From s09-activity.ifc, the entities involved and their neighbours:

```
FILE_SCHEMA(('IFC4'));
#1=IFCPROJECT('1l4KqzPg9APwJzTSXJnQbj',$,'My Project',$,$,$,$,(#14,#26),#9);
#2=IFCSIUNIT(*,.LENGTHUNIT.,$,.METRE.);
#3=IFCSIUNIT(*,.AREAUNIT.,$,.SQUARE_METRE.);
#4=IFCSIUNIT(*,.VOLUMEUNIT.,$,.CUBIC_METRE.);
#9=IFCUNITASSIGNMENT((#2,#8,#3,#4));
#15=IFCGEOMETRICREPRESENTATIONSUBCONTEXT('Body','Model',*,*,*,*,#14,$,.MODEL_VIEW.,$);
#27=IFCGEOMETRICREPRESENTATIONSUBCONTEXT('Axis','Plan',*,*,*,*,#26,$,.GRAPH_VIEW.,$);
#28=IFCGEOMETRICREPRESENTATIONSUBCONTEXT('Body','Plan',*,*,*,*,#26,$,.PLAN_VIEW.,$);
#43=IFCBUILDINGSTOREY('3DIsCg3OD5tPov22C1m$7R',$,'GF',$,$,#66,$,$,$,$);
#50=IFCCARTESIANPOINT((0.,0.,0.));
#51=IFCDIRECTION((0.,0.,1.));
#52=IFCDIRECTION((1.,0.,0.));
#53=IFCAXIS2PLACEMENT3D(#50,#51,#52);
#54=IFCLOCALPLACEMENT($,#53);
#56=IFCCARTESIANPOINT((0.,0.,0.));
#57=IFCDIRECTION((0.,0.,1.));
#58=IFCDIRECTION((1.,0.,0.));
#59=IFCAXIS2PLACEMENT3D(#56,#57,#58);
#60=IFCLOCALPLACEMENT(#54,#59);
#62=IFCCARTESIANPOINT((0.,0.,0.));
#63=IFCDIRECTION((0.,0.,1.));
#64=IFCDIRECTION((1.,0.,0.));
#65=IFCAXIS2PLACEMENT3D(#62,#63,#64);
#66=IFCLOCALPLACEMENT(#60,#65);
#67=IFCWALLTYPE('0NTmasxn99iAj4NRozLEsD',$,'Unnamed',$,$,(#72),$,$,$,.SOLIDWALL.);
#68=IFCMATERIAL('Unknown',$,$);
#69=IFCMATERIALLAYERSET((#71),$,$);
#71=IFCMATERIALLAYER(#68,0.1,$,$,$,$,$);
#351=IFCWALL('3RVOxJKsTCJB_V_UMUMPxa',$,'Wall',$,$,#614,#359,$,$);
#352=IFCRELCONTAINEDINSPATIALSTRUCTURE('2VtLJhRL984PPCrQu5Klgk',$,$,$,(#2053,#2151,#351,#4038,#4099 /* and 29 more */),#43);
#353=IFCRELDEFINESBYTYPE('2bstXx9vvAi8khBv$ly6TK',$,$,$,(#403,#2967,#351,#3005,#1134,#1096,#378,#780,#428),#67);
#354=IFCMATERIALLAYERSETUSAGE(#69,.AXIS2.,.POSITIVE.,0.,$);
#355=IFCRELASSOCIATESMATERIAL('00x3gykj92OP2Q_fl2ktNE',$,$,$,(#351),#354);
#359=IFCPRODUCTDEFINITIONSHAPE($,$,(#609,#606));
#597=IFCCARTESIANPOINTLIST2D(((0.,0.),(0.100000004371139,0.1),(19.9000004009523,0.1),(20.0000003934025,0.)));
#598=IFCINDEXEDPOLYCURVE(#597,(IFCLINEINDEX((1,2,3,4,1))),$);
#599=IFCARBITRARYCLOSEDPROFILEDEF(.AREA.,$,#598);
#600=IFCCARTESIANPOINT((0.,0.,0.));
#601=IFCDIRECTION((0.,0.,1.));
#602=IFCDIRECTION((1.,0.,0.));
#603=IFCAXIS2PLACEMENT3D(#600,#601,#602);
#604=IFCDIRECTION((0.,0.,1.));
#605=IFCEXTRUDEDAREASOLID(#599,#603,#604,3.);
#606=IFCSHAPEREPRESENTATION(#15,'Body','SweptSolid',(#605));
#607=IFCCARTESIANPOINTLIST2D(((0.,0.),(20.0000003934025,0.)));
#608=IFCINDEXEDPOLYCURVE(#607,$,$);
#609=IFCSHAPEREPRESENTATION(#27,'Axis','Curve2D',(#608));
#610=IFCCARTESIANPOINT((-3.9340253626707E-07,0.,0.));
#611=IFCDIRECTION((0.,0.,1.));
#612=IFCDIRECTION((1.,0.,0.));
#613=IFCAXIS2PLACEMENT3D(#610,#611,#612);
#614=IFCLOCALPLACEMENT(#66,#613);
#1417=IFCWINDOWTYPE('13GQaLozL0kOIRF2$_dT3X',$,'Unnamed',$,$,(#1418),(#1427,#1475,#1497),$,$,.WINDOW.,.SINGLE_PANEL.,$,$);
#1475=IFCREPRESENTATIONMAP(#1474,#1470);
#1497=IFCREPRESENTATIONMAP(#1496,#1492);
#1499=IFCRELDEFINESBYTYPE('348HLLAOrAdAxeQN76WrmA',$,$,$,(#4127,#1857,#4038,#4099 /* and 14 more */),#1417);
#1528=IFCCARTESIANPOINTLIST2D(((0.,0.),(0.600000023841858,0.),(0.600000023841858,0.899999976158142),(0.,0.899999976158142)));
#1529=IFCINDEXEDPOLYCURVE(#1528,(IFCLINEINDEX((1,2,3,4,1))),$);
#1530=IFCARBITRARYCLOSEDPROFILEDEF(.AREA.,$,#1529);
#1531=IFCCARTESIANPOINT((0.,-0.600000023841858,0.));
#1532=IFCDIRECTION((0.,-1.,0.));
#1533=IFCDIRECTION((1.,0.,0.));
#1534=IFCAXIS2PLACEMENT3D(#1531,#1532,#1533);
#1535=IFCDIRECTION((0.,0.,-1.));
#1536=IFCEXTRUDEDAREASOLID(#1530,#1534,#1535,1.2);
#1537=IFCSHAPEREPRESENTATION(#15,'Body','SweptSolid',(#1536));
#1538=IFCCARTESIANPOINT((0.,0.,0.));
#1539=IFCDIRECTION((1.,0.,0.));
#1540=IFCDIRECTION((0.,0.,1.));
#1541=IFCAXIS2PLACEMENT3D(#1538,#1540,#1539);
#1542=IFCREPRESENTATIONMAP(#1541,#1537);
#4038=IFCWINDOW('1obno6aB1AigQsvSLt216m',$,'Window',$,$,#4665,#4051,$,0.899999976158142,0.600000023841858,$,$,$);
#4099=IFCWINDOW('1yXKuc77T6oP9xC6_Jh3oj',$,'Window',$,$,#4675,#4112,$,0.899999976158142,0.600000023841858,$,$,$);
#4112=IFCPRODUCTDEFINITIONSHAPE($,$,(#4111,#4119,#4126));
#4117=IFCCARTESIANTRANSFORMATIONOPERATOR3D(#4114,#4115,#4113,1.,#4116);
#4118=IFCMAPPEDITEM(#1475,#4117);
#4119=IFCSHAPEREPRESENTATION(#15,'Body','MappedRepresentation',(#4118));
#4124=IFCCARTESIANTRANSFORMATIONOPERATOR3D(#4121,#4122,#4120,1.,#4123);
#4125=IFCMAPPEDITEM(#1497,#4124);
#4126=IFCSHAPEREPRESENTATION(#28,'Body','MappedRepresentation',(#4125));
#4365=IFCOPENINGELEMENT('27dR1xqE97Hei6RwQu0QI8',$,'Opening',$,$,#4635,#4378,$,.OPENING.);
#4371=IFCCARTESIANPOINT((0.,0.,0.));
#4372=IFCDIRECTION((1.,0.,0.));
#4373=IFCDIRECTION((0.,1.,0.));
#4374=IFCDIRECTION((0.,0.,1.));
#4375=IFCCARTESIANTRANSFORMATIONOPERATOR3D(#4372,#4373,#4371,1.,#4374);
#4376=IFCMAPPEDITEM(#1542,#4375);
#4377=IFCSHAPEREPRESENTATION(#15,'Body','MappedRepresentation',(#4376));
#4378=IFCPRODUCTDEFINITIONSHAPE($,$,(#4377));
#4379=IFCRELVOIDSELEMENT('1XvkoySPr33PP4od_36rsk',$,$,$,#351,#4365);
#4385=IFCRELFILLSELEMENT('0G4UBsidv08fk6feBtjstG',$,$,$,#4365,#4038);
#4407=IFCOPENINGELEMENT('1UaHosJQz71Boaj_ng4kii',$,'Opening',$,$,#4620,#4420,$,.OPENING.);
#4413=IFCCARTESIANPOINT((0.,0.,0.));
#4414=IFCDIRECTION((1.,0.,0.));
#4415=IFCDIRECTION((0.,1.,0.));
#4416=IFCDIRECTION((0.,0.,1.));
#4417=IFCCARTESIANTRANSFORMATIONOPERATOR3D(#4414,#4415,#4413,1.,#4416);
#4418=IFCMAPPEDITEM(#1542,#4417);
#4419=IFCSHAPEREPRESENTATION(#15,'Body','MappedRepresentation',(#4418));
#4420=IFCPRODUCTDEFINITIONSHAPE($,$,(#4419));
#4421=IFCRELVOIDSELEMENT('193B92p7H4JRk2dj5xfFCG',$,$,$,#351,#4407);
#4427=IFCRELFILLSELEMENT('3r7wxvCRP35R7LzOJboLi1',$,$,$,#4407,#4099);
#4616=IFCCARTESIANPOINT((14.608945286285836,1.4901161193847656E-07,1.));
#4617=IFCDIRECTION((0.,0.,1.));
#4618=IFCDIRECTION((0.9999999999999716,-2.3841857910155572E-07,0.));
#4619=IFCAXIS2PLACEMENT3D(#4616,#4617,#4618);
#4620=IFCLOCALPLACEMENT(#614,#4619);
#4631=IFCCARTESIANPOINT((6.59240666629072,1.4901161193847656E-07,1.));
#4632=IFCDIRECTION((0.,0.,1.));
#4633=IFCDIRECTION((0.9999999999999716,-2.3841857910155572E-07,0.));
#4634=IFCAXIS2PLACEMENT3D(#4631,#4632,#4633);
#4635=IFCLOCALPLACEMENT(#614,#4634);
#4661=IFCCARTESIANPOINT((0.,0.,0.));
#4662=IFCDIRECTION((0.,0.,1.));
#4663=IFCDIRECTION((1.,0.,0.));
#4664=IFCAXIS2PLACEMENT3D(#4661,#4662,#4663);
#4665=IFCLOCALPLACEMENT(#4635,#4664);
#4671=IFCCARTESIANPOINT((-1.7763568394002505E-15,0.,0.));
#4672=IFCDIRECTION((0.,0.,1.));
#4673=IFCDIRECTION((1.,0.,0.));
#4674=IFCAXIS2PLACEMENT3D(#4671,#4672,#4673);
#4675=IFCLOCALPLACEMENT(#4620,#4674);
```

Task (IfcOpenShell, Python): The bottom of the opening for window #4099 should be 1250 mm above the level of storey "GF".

```python
import numpy as np
import ifcopenshell
import ifcopenshell.api.geometry
import ifcopenshell.geom
import ifcopenshell.util.element
import ifcopenshell.util.placement
import ifcopenshell.util.shape
import ifcopenshell.util.unit

model = ifcopenshell.open("s09-activity.ifc")
unit_scale = ifcopenshell.util.unit.calculate_unit_scale(model)

window = model.by_id(4099)
opening = window.FillsVoids[0].RelatingOpeningElement
storey = ifcopenshell.util.element.get_container(window, ifc_class="IfcBuildingStorey")
level = ifcopenshell.util.placement.get_local_placement(storey.ObjectPlacement)[2, 3]

# The opening's origin need not be at the sill, so measure its lowest point.
shape = ifcopenshell.geom.create_shape(ifcopenshell.geom.settings(), opening)
bottom = ifcopenshell.util.shape.get_shape_bottom_elevation(shape, shape.geometry) / unit_scale
dz = level + 1.25 / unit_scale - bottom

shift = np.array([0.0, 0.0, dz])
# The window is placed relative to its opening, so it follows when the opening moves.
matrix = ifcopenshell.util.placement.get_local_placement(opening.ObjectPlacement)
matrix[:3, 3] += shift
ifcopenshell.api.geometry.edit_object_placement(
    model, product=opening, matrix=matrix, is_si=False, should_transform_children=True
)

print(f"moved by {dz * unit_scale:+.3f} m")

model.write("s09-activity_v2.ifc")
```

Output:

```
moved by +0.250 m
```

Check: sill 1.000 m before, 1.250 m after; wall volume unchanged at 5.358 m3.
